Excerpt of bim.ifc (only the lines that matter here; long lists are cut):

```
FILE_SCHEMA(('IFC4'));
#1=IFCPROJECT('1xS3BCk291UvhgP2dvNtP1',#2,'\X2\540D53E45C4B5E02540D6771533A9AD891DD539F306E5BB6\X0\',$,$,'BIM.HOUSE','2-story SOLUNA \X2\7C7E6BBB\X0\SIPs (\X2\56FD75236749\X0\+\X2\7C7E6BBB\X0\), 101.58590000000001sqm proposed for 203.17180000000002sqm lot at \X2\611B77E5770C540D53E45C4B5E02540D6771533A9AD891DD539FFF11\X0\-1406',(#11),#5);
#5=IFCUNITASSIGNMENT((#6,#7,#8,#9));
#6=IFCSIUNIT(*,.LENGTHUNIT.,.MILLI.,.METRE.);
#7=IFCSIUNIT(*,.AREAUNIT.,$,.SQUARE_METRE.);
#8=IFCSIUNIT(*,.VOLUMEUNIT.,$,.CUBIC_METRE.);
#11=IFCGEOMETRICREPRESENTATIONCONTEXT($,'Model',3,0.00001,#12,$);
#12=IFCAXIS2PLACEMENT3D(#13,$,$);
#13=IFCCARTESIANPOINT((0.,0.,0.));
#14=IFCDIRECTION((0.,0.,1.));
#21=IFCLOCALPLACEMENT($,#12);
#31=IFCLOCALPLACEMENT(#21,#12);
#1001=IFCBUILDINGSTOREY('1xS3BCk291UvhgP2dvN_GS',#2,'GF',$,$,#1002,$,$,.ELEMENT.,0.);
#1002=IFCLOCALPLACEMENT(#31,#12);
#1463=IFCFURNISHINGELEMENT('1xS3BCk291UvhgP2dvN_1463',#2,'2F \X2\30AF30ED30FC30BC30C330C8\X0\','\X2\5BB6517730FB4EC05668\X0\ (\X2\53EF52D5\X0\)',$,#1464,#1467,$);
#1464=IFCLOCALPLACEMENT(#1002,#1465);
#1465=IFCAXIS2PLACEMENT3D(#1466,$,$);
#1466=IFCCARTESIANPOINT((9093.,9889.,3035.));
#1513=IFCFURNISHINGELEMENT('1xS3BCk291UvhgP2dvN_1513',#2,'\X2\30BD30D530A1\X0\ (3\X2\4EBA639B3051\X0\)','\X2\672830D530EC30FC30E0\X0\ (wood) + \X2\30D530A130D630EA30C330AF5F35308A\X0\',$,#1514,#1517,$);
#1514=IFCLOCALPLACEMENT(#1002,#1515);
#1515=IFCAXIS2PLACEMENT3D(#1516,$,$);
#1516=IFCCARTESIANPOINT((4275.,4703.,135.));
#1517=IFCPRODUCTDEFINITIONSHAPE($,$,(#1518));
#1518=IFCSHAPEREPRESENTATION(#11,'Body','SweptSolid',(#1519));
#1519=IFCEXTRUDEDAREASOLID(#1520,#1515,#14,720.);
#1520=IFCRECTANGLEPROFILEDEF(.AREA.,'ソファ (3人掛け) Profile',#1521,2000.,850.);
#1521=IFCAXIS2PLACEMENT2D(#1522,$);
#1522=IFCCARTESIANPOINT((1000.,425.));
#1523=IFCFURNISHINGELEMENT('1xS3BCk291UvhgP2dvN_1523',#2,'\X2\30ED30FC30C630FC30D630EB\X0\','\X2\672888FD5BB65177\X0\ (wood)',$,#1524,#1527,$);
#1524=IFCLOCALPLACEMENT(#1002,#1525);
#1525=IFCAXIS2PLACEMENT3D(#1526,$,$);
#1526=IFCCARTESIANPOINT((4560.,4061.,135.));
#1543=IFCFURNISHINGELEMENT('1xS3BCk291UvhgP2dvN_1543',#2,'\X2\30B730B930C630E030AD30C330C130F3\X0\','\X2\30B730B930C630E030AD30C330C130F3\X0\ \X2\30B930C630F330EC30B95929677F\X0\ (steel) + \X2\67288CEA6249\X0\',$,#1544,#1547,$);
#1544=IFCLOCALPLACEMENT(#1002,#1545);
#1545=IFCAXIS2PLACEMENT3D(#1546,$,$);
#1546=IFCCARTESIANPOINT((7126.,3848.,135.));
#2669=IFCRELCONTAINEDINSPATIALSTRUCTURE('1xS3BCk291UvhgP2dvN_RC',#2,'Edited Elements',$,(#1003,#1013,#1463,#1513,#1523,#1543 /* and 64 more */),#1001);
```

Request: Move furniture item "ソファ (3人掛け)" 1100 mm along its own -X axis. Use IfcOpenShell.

```python
import ifcopenshell
import ifcopenshell.api.geometry
import ifcopenshell.util.placement
import ifcopenshell.util.unit

model = ifcopenshell.open("bim.ifc")
unit_scale = ifcopenshell.util.unit.calculate_unit_scale(model)

item = model.by_guid("1xS3BCk291UvhgP2dvN_1513")
matrix = ifcopenshell.util.placement.get_local_placement(item.ObjectPlacement)
matrix[:3, 3] -= matrix[:3, 0] * 1.1 / unit_scale
ifcopenshell.api.geometry.edit_object_placement(model, product=item, matrix=matrix, is_si=False)

print(ifcopenshell.util.placement.get_local_placement(item.ObjectPlacement).round(3) + 0.0)

model.write("bim_v2.ifc")
```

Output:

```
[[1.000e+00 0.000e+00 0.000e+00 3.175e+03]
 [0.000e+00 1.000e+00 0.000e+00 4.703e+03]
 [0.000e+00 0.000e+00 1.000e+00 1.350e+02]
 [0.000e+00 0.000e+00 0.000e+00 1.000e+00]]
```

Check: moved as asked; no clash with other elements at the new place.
